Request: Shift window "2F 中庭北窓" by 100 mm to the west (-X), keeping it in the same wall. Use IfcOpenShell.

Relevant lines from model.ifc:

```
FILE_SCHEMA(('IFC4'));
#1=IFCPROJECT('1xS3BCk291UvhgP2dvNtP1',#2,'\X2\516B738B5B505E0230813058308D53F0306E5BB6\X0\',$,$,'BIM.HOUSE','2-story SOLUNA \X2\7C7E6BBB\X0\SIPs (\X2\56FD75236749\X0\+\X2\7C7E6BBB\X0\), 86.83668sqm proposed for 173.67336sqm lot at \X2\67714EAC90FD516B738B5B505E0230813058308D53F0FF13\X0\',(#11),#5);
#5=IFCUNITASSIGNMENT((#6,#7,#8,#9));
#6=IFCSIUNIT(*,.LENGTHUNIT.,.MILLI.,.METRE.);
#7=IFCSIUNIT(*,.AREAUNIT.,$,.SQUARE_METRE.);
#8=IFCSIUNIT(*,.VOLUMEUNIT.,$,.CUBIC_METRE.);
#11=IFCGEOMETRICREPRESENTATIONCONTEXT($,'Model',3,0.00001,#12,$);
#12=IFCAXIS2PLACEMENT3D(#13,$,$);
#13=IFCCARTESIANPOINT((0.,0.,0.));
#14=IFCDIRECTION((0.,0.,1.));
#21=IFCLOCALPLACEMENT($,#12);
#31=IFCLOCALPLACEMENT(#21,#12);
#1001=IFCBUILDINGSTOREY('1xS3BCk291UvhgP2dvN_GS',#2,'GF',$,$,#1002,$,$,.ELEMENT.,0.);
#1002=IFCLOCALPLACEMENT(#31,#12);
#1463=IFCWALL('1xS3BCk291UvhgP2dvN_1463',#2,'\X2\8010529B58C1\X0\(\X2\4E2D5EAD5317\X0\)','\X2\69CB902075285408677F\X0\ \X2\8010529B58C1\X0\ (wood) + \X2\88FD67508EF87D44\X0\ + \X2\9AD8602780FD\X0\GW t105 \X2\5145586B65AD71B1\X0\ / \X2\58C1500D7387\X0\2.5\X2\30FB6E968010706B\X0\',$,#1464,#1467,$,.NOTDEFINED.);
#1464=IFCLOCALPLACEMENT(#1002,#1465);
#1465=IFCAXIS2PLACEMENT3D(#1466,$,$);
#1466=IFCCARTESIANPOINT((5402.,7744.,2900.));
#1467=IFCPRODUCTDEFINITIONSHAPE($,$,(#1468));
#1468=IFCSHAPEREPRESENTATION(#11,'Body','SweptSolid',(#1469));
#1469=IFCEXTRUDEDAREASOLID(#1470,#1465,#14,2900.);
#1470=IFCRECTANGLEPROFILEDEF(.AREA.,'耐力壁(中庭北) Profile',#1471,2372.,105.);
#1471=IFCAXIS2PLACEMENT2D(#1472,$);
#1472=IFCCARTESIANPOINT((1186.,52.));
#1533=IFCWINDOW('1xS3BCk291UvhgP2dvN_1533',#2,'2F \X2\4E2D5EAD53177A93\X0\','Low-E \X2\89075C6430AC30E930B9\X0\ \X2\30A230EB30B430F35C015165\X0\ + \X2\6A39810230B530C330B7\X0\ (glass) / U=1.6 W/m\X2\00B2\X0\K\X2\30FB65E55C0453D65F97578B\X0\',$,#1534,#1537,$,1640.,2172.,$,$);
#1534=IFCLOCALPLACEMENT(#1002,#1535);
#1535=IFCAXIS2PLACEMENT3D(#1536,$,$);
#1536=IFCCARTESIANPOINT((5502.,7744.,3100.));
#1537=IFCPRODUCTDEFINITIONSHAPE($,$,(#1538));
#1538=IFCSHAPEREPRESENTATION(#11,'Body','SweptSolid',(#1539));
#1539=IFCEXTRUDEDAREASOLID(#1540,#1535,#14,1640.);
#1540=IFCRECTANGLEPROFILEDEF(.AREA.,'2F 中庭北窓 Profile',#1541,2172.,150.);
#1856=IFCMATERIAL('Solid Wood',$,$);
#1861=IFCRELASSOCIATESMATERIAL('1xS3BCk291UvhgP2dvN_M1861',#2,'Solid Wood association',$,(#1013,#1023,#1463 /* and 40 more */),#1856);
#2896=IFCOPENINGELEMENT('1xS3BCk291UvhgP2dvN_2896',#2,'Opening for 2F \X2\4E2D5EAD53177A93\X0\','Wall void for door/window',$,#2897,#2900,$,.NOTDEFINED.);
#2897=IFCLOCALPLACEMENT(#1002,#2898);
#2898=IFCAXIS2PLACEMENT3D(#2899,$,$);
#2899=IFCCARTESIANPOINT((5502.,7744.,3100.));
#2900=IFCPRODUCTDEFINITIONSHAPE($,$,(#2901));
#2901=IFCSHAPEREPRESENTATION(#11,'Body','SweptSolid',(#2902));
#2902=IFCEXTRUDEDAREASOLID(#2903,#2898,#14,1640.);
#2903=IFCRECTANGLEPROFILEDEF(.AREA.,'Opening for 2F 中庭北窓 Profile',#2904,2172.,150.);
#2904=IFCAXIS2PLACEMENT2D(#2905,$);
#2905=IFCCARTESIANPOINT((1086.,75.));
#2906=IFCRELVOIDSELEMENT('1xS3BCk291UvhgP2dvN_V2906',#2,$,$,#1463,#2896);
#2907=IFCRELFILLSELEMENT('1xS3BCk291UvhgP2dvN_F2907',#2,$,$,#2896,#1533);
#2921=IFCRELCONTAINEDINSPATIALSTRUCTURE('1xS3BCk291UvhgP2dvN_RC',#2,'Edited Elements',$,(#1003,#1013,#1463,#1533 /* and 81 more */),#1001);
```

```python
import ifcopenshell
import ifcopenshell.api.geometry
import ifcopenshell.util.placement
import ifcopenshell.util.unit

model = ifcopenshell.open("model.ifc")
unit_scale = ifcopenshell.util.unit.calculate_unit_scale(model)

window = model.by_id(1533)
opening = window.FillsVoids[0].RelatingOpeningElement
wall = opening.VoidsElements[0].RelatingBuildingElement

wall_matrix = ifcopenshell.util.placement.get_local_placement(wall.ObjectPlacement)
shift = wall_matrix[:3, 0] * -0.1 / unit_scale
before = ifcopenshell.util.placement.get_local_placement(window.ObjectPlacement)[:3, 3].copy()

# The window is not placed relative to its opening, so move both.
for product in (opening, window):
    matrix = ifcopenshell.util.placement.get_local_placement(product.ObjectPlacement)
    matrix[:3, 3] += shift
    ifcopenshell.api.geometry.edit_object_placement(model, product=product, matrix=matrix, is_si=False)

after = ifcopenshell.util.placement.get_local_placement(window.ObjectPlacement)[:3, 3]
print("window moved by", (after - before).round(3) + 0.0)

model.write("model_v2.ifc")
```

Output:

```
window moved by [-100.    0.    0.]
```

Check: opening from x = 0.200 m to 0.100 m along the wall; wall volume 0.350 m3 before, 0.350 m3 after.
